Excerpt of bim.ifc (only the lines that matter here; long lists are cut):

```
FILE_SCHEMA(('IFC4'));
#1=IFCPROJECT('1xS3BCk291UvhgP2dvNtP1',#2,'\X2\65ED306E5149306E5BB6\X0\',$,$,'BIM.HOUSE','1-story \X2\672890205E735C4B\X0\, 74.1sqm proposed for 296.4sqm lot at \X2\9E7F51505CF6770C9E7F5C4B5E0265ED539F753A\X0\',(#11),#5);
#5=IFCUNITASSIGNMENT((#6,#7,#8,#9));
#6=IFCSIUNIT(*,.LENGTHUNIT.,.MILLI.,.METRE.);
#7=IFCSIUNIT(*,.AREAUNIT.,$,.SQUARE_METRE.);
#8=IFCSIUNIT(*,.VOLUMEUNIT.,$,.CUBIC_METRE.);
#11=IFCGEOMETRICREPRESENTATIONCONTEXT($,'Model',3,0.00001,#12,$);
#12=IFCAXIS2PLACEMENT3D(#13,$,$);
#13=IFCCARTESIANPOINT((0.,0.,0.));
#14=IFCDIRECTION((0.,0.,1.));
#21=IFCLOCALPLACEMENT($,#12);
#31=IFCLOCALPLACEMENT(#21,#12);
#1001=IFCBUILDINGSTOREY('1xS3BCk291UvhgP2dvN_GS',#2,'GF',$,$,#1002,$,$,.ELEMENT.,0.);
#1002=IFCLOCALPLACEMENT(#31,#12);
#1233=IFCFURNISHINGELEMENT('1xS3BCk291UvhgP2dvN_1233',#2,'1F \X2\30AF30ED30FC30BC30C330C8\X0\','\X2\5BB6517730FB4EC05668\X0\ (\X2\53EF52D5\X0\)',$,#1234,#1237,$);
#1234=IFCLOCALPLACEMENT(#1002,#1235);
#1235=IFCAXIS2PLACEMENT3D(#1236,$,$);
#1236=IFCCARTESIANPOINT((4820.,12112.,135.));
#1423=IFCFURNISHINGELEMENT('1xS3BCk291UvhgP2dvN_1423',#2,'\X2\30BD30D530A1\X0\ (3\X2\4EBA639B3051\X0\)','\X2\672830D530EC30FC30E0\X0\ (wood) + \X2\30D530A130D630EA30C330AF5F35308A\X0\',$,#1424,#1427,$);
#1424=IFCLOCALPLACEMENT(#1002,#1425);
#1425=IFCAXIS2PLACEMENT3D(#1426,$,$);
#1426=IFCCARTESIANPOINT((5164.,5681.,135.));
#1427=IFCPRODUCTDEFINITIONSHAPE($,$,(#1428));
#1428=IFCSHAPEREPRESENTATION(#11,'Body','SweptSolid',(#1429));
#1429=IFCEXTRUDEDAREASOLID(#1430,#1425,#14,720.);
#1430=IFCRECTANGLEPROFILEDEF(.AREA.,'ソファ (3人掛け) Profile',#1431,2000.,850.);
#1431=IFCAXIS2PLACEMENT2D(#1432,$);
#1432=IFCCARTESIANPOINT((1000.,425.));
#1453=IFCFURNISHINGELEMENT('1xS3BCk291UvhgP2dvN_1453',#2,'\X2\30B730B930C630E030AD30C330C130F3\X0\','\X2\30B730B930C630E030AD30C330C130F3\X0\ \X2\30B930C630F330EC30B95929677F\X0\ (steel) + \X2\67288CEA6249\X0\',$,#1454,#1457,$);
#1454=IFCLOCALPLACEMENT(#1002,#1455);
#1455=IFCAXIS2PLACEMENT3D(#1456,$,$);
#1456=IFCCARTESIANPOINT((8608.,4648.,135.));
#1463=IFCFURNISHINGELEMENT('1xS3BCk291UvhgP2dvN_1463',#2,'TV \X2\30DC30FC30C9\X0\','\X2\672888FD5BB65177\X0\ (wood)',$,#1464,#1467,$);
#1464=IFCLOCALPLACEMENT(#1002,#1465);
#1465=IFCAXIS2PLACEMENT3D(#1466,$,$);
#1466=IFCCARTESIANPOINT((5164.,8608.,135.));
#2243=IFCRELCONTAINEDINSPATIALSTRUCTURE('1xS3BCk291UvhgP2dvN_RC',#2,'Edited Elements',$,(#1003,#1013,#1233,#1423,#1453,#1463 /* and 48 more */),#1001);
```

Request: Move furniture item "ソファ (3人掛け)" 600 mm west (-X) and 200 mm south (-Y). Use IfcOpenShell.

```python
import ifcopenshell
import ifcopenshell.api.geometry
import ifcopenshell.util.placement
import ifcopenshell.util.unit

model = ifcopenshell.open("bim.ifc")
unit_scale = ifcopenshell.util.unit.calculate_unit_scale(model)

item = model.by_guid("1xS3BCk291UvhgP2dvN_1423")
matrix = ifcopenshell.util.placement.get_local_placement(item.ObjectPlacement)
matrix[0, 3] -= 0.6 / unit_scale
matrix[1, 3] -= 0.2 / unit_scale
ifcopenshell.api.geometry.edit_object_placement(model, product=item, matrix=matrix, is_si=False)

print(ifcopenshell.util.placement.get_local_placement(item.ObjectPlacement).round(3) + 0.0)

model.write("bim_edited.ifc")
```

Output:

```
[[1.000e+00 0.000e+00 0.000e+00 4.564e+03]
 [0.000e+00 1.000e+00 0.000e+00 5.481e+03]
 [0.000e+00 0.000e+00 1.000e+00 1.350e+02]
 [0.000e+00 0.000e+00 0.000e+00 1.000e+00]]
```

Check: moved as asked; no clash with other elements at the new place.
